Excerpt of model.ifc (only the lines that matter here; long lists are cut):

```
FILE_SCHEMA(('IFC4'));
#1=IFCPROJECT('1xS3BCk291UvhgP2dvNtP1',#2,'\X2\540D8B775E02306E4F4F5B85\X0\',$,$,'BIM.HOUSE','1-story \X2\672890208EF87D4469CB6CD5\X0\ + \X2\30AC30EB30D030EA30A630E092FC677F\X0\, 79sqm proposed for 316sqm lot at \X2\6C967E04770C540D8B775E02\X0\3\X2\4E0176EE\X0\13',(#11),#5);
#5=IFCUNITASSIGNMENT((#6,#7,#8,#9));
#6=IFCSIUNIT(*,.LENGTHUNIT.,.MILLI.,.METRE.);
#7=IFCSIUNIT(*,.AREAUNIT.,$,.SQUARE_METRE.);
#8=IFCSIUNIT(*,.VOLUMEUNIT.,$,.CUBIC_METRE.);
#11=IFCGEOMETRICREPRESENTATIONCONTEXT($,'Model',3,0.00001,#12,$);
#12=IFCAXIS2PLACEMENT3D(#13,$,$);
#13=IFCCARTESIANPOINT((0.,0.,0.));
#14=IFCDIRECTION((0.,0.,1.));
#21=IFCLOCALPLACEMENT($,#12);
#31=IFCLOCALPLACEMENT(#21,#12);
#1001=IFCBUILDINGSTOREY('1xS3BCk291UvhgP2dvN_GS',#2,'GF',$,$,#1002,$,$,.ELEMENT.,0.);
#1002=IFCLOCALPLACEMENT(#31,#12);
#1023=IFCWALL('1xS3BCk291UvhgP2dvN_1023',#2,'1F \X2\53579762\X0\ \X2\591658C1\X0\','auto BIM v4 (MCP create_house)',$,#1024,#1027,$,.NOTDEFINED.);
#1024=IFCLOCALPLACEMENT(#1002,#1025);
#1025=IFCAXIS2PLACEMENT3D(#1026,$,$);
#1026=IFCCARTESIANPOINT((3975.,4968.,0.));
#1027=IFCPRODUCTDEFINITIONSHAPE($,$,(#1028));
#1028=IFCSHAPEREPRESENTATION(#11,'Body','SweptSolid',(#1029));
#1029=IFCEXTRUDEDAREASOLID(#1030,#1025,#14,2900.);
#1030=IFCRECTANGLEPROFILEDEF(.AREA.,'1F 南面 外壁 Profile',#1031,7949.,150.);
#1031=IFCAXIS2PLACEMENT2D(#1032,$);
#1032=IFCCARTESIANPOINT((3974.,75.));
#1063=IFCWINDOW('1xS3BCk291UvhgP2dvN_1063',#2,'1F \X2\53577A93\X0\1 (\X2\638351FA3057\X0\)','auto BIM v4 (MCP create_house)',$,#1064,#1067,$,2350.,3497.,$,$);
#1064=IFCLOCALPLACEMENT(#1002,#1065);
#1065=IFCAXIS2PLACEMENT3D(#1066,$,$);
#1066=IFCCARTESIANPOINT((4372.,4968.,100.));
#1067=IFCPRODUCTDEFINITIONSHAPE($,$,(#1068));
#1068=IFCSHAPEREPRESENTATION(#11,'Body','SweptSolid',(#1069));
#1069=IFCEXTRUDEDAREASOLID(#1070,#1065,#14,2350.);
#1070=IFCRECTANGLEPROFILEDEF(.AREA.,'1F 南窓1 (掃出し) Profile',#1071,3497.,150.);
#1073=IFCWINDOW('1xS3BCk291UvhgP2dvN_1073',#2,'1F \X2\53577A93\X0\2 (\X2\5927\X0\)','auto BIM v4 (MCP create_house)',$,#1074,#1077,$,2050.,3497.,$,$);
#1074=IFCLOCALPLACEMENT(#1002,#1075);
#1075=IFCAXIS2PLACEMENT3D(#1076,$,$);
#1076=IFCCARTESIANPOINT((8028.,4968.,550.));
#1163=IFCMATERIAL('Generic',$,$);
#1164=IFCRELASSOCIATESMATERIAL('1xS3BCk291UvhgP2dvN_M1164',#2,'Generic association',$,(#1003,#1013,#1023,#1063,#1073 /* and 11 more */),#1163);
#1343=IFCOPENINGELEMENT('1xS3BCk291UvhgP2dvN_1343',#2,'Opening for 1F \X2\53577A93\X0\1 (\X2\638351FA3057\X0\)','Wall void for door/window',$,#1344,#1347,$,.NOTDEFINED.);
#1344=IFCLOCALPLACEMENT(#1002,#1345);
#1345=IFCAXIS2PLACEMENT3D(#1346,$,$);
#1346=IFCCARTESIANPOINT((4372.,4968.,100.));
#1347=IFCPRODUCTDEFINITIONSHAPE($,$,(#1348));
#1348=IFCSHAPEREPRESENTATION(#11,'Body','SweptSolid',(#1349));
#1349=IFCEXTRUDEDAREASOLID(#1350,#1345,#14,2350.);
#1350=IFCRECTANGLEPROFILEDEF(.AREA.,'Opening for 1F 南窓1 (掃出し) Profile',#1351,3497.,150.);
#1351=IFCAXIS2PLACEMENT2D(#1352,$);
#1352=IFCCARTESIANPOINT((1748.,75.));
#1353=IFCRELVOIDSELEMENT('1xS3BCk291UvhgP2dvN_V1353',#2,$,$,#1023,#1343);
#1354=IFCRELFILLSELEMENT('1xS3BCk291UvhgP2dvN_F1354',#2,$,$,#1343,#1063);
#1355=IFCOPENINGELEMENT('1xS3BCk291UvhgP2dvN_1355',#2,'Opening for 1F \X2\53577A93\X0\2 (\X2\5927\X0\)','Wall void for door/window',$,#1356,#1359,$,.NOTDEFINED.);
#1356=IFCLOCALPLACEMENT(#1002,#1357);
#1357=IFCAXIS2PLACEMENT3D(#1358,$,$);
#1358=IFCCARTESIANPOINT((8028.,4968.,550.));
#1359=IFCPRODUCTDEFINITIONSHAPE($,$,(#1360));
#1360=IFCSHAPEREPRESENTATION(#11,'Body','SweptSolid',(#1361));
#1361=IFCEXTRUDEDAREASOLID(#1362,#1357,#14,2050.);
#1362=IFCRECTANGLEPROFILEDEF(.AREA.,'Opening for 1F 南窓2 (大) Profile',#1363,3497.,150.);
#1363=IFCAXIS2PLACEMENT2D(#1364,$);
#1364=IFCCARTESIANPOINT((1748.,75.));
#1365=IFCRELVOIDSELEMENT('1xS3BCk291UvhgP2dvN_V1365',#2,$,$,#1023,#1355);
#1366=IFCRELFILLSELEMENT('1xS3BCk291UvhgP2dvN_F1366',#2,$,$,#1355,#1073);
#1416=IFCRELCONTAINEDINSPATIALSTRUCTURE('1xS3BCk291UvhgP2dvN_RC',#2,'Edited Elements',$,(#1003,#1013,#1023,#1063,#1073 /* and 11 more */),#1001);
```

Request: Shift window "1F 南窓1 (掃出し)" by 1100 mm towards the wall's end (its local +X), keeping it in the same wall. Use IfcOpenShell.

```python
import ifcopenshell
import ifcopenshell.api.geometry
import ifcopenshell.util.placement
import ifcopenshell.util.unit

model = ifcopenshell.open("model.ifc")
unit_scale = ifcopenshell.util.unit.calculate_unit_scale(model)

window = model.by_guid("1xS3BCk291UvhgP2dvN_1063")
opening = window.FillsVoids[0].RelatingOpeningElement
wall = opening.VoidsElements[0].RelatingBuildingElement

wall_matrix = ifcopenshell.util.placement.get_local_placement(wall.ObjectPlacement)
shift = wall_matrix[:3, 0] * 1.1 / unit_scale
before = ifcopenshell.util.placement.get_local_placement(window.ObjectPlacement)[:3, 3].copy()

# The window is not placed relative to its opening, so move both.
for product in (opening, window):
    matrix = ifcopenshell.util.placement.get_local_placement(product.ObjectPlacement)
    matrix[:3, 3] += shift
    ifcopenshell.api.geometry.edit_object_placement(model, product=product, matrix=matrix, is_si=False)

after = ifcopenshell.util.placement.get_local_placement(window.ObjectPlacement)[:3, 3]
print("window moved by", (after - before).round(3) + 0.0)

model.write("model_rev.ifc")
```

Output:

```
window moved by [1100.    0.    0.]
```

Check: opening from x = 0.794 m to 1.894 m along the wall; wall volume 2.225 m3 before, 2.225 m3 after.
